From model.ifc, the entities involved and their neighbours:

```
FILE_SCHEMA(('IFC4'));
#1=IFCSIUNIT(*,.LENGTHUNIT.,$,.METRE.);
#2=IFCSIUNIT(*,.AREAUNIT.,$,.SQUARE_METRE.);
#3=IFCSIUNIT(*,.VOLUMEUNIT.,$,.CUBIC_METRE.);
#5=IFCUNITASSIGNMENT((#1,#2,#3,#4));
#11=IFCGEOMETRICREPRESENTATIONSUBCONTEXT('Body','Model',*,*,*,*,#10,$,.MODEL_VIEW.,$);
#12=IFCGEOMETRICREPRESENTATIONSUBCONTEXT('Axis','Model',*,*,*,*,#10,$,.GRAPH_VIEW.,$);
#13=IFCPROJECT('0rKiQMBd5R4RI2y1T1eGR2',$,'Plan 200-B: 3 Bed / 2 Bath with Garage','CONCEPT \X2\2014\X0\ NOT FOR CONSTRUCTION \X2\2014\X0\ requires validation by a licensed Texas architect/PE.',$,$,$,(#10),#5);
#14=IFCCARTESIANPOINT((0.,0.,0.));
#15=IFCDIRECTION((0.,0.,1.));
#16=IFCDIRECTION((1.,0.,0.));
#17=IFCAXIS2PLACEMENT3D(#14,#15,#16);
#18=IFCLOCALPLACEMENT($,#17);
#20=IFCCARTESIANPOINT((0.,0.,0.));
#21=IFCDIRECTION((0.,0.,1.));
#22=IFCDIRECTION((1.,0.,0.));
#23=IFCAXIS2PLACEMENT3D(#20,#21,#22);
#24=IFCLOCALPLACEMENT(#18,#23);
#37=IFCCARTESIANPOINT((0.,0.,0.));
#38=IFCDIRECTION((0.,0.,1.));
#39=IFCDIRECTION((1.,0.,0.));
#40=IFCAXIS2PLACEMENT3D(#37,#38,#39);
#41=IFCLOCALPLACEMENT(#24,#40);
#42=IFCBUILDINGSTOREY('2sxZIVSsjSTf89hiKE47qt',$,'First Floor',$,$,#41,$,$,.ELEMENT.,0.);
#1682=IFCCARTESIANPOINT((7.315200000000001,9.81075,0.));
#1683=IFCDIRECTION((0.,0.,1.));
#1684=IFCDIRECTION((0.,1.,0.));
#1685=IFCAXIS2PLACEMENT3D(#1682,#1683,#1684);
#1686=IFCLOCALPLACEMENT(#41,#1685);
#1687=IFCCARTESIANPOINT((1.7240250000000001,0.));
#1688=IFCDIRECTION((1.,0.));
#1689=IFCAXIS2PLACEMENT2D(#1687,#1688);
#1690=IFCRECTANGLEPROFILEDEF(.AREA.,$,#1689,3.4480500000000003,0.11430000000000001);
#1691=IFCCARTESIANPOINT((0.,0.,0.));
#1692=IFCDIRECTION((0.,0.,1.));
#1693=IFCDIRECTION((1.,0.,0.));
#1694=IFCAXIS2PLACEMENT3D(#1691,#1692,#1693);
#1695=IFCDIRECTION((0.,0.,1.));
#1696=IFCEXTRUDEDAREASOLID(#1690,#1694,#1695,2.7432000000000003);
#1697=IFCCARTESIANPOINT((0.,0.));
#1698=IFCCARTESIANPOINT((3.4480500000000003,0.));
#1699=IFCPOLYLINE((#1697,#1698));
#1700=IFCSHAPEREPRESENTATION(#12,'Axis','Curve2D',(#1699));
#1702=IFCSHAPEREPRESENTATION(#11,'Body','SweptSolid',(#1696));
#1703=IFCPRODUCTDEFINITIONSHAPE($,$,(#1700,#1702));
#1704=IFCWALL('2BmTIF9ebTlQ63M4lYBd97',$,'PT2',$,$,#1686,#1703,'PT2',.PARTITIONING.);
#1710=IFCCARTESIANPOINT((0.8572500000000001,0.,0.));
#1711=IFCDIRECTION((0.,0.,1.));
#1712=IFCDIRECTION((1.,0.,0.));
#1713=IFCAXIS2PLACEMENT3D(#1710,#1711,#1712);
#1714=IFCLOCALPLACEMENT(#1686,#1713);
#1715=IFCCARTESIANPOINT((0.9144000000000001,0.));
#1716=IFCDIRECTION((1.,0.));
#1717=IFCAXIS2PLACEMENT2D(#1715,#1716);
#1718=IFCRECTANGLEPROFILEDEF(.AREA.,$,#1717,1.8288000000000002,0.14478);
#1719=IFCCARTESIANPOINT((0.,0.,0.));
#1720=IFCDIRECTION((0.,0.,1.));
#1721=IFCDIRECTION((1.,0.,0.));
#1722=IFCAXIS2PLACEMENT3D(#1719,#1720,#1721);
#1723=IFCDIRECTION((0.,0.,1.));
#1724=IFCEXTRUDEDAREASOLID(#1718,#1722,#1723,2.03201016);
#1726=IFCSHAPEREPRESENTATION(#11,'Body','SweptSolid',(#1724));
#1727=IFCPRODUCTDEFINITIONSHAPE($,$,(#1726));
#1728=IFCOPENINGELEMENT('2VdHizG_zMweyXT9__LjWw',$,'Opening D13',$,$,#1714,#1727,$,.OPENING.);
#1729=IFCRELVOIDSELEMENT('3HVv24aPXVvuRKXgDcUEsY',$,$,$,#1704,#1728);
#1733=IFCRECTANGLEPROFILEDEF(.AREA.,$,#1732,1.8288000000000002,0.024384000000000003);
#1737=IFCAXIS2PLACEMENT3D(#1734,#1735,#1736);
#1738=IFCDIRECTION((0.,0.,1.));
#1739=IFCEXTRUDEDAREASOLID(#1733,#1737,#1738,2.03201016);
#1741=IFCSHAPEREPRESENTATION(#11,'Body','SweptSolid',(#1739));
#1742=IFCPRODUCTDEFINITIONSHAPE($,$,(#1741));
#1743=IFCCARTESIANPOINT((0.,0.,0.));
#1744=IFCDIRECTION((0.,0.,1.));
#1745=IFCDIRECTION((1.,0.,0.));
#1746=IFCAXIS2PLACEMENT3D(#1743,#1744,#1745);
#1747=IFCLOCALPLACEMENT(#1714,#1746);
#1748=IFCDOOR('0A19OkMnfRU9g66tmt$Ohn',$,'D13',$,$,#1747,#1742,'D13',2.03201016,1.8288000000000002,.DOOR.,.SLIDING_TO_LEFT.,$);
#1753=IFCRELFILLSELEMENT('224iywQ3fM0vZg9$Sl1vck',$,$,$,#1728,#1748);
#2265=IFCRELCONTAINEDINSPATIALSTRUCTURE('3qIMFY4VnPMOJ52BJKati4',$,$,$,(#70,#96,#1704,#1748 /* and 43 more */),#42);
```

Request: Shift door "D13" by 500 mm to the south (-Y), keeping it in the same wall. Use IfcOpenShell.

```python
import ifcopenshell
import ifcopenshell.api.geometry
import ifcopenshell.util.placement
import ifcopenshell.util.unit

model = ifcopenshell.open("model.ifc")
unit_scale = ifcopenshell.util.unit.calculate_unit_scale(model)

door = model.by_id(1748)
opening = door.FillsVoids[0].RelatingOpeningElement
wall = opening.VoidsElements[0].RelatingBuildingElement

wall_matrix = ifcopenshell.util.placement.get_local_placement(wall.ObjectPlacement)
shift = wall_matrix[:3, 0] * -0.5 / unit_scale
before = ifcopenshell.util.placement.get_local_placement(door.ObjectPlacement)[:3, 3].copy()

# The door is placed relative to its opening, so it follows when the opening moves.
matrix = ifcopenshell.util.placement.get_local_placement(opening.ObjectPlacement)
matrix[:3, 3] += shift
ifcopenshell.api.geometry.edit_object_placement(
    model, product=opening, matrix=matrix, is_si=False, should_transform_children=True
)

after = ifcopenshell.util.placement.get_local_placement(door.ObjectPlacement)[:3, 3]
print("door moved by", (after - before).round(3) + 0.0)

model.write("model_edited.ifc")
```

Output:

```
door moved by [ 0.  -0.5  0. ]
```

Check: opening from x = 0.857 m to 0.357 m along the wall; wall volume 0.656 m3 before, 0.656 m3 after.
